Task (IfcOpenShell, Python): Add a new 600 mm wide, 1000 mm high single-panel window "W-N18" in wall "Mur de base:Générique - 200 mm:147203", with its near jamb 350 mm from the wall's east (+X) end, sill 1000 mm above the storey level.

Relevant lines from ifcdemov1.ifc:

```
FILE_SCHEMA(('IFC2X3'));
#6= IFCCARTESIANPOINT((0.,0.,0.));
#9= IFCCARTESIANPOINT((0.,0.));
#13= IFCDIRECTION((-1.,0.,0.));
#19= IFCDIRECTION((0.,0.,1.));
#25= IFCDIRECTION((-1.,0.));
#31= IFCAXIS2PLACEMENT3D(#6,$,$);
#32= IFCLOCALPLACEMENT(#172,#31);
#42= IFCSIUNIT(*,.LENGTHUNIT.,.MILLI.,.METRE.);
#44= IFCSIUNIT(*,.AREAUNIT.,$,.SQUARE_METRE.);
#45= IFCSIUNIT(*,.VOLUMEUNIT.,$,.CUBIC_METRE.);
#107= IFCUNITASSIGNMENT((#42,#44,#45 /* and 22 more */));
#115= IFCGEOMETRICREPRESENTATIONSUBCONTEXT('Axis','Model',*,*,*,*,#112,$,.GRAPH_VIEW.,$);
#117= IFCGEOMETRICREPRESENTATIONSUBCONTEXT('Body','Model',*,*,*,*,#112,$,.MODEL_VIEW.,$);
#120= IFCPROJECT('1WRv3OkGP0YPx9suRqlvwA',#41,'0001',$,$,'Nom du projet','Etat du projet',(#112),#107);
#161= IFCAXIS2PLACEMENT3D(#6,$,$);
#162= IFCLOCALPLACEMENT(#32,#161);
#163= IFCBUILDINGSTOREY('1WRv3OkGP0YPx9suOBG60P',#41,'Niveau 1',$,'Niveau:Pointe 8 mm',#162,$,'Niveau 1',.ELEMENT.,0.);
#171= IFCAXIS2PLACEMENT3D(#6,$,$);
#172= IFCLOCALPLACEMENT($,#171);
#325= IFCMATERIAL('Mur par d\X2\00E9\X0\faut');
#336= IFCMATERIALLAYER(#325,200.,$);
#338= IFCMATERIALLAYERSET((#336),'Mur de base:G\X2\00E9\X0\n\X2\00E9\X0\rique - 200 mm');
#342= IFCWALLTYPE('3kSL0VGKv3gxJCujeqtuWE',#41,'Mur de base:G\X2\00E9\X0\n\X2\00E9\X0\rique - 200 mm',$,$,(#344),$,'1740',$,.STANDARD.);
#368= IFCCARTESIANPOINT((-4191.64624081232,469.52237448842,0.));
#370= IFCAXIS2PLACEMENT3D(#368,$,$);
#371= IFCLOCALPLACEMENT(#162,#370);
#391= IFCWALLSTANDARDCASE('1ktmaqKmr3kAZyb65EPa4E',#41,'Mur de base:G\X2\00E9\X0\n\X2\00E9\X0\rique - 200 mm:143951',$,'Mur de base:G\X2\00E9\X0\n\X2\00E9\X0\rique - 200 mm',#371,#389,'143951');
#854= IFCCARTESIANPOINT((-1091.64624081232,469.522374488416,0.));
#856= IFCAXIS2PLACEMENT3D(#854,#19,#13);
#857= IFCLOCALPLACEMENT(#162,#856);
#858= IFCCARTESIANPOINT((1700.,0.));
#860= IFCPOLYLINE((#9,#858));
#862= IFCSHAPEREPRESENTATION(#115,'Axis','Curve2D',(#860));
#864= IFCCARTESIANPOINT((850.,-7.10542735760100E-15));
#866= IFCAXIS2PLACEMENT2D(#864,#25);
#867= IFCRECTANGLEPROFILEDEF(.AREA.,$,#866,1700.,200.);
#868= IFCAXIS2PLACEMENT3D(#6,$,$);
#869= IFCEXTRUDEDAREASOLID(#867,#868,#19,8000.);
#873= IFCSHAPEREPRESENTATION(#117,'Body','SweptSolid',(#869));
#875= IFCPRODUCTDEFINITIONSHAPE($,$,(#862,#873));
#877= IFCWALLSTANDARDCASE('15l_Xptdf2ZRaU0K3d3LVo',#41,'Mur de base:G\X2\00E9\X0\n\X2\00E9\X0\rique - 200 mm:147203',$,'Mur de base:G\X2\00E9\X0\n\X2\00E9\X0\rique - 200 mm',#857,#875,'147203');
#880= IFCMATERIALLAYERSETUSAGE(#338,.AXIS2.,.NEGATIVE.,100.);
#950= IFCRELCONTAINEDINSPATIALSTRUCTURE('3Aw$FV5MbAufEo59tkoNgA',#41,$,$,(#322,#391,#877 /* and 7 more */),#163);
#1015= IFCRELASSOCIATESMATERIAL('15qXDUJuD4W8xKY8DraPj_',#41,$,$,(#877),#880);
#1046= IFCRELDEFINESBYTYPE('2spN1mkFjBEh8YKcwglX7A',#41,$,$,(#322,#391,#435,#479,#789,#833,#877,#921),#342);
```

```python
import numpy as np
import ifcopenshell
import ifcopenshell.api.feature
import ifcopenshell.api.geometry
import ifcopenshell.api.root
import ifcopenshell.api.spatial
import ifcopenshell.api.type
import ifcopenshell.geom
import ifcopenshell.util.element
import ifcopenshell.util.placement
import ifcopenshell.util.representation
import ifcopenshell.util.shape
import ifcopenshell.util.unit

model = ifcopenshell.open("ifcdemov1.ifc")
unit_scale = ifcopenshell.util.unit.calculate_unit_scale(model)
settings = ifcopenshell.geom.settings()


def volume(element):
    """Net volume in cubic metres, openings subtracted."""
    shape = ifcopenshell.geom.create_shape(settings, element)
    return ifcopenshell.util.shape.get_volume(shape.geometry)


wall = model.by_guid("15l_Xptdf2ZRaU0K3d3LVo")
storey = ifcopenshell.util.element.get_container(wall, ifc_class="IfcBuildingStorey")
context = ifcopenshell.util.representation.get_context(model, "Model", "Body", "MODEL_VIEW")
before = volume(wall)

width, height, from_end, sill = 0.6, 1, 0.35, 1  # metres

# The wall runs along its own X axis, and the end named is its -X end.
wall_shape = ifcopenshell.geom.create_shape(settings, wall)
x, y, z = ifcopenshell.util.shape.get_vertices(wall_shape.geometry).T
start = x.min() + from_end
face, thickness = float(y.min()), float(y.max() - y.min())
wall_matrix = ifcopenshell.util.placement.get_local_placement(wall.ObjectPlacement)
level = ifcopenshell.util.placement.get_local_placement(storey.ObjectPlacement)[2, 3]


def in_wall(x, y):
    """Placement at x, y metres in the wall's axes, at sill height."""
    matrix = wall_matrix.copy()
    matrix[:, 3] = wall_matrix @ np.array([x / unit_scale, y / unit_scale, 0.0, 1.0])
    matrix[2, 3] = level + sill / unit_scale
    return matrix


# Opening: a box that overshoots both wall faces by 50 mm.
opening = ifcopenshell.api.root.create_entity(model, ifc_class="IfcOpeningElement")
box = ifcopenshell.api.geometry.add_wall_representation(
    model, context=context, length=width, height=height, thickness=thickness + 0.1
)
ifcopenshell.api.geometry.assign_representation(model, product=opening, representation=box)
ifcopenshell.api.geometry.edit_object_placement(model, product=opening, matrix=in_wall(start, face - 0.05), is_si=False)
ifcopenshell.api.feature.add_feature(model, feature=opening, element=wall)

window = ifcopenshell.api.root.create_entity(model, ifc_class="IfcWindow", name="W-N18")
window.OverallWidth, window.OverallHeight = width / unit_scale, height / unit_scale
body = ifcopenshell.api.geometry.add_window_representation(
    model,
    context=context,
    overall_width=window.OverallWidth,
    overall_height=window.OverallHeight,
    partition_type="SINGLE_PANEL",
)
ifcopenshell.api.geometry.assign_representation(model, product=window, representation=body)
ifcopenshell.api.spatial.assign_container(model, products=[window], relating_structure=storey)
fills = ifcopenshell.api.feature.add_filling(model, opening=opening, element=window)
fills.OwnerHistory = window.OwnerHistory  # required in IFC2X3

# IFC2X3 keeps the operation on the window style.
style = ifcopenshell.api.root.create_entity(model, ifc_class="IfcWindowStyle", name="W-N18")
style.OperationType, style.ConstructionType = "SINGLE_PANEL", "NOTDEFINED"
style.ParameterTakesPrecedence = style.Sizeable = False
ifcopenshell.api.type.assign_type(model, related_objects=[window], relating_type=style)

# Centre the window in the wall's thickness.
ifcopenshell.api.geometry.edit_object_placement(model, product=window, matrix=in_wall(start, face), is_si=False)
window_shape = ifcopenshell.geom.create_shape(settings, window)
depth = ifcopenshell.util.shape.get_vertices(window_shape.geometry)[:, 1]
offset = face + thickness / 2 - (depth.min() + depth.max()) / 2
ifcopenshell.api.geometry.edit_object_placement(model, product=window, matrix=in_wall(start, offset), is_si=False)

after = volume(wall)

print(f"wall volume {before:.3f} -> {after:.3f} m3")

model.write("ifcdemov1_updated.ifc")
```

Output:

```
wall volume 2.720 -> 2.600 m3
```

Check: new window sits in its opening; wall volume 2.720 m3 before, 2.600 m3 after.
